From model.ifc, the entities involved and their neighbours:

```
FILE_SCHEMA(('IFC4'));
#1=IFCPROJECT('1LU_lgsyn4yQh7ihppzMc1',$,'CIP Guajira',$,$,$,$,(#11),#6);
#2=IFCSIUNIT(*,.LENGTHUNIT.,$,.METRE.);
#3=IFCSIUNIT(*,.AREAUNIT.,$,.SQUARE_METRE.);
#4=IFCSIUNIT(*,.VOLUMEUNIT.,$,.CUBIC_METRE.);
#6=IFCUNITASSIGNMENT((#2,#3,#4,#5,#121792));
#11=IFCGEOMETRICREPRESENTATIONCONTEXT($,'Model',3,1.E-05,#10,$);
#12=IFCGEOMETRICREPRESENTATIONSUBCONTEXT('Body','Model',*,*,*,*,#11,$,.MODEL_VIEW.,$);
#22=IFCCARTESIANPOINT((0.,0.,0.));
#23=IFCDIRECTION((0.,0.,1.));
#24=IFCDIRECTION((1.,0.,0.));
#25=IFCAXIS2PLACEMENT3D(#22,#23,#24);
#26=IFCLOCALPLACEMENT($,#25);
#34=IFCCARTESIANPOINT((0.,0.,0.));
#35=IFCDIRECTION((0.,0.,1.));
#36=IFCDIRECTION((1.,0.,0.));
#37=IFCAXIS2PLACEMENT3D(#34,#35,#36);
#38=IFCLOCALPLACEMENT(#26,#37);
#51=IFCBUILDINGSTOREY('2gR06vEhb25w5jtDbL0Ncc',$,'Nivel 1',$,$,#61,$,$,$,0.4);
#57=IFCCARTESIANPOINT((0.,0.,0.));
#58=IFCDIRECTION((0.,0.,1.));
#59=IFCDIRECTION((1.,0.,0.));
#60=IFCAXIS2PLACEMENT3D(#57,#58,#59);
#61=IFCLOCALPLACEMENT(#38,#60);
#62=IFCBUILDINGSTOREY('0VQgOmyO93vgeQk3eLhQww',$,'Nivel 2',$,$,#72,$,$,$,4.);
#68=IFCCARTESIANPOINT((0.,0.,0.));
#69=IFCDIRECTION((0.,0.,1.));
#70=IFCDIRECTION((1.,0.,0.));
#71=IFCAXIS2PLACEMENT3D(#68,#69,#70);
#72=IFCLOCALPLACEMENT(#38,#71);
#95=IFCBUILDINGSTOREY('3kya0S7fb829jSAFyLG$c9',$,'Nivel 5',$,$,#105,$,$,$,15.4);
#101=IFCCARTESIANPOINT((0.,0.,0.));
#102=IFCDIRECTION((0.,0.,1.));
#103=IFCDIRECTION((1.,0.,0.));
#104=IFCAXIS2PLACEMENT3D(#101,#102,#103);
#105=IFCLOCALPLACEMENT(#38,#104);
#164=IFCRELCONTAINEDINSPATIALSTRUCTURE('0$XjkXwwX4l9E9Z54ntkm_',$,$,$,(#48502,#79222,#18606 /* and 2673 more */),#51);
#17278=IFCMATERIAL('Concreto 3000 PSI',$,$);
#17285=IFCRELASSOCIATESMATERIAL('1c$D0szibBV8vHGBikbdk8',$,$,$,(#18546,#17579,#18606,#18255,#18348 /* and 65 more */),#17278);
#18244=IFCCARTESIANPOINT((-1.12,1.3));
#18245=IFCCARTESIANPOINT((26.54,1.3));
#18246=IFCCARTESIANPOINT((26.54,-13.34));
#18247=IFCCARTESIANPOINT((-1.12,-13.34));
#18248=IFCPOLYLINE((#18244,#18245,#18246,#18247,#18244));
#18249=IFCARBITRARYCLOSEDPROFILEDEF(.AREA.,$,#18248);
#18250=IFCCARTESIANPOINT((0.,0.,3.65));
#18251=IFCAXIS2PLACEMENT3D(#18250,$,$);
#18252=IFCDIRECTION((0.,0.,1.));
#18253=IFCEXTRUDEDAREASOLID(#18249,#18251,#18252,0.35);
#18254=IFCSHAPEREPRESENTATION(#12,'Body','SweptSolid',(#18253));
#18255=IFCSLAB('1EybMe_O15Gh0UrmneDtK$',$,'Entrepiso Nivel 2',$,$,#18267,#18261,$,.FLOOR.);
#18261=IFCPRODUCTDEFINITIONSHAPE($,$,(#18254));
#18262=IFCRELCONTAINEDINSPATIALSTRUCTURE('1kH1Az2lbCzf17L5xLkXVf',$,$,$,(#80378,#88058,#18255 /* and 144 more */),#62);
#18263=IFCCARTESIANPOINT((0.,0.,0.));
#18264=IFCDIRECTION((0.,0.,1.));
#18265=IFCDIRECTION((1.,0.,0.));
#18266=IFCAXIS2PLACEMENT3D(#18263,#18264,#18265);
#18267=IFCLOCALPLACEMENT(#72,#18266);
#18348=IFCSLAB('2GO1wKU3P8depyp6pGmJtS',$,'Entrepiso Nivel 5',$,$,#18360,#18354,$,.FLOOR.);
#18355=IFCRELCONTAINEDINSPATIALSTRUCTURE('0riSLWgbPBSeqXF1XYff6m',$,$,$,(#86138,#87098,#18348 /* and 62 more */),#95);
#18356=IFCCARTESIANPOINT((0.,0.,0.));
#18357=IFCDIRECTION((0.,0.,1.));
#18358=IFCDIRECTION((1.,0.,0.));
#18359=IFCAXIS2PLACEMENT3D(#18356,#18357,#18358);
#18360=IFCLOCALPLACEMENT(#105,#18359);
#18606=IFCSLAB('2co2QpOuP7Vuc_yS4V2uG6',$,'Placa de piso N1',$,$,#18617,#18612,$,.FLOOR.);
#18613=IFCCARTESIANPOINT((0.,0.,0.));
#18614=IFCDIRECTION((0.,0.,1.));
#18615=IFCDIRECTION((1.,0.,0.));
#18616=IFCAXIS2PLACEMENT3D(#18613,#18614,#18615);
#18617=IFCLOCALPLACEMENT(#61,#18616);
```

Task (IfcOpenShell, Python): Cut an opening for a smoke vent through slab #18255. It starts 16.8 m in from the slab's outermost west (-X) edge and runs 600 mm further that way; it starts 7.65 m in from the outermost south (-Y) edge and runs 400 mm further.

```python
import numpy as np
import ifcopenshell
import ifcopenshell.api.feature
import ifcopenshell.api.geometry
import ifcopenshell.api.root
import ifcopenshell.geom
import ifcopenshell.util.placement
import ifcopenshell.util.representation
import ifcopenshell.util.shape
import ifcopenshell.util.unit

model = ifcopenshell.open("model.ifc")
unit_scale = ifcopenshell.util.unit.calculate_unit_scale(model)
settings = ifcopenshell.geom.settings()


def volume(element):
    """Net volume in cubic metres, openings subtracted."""
    shape = ifcopenshell.geom.create_shape(settings, element)
    return ifcopenshell.util.shape.get_volume(shape.geometry)


slab = model.by_id(18255)
before = volume(slab)

# Extent in the slab's own axes, in metres. The edges named are its -X and -Y sides.
slab_shape = ifcopenshell.geom.create_shape(settings, slab)
vertices = ifcopenshell.util.shape.get_vertices(slab_shape.geometry)
x_min, y_min, bottom = vertices.min(axis=0)
top = vertices[:, 2].max()

opening = ifcopenshell.api.root.create_entity(model, ifc_class="IfcOpeningElement", name="Smoke vent opening", predefined_type="OPENING")
context = ifcopenshell.util.representation.get_context(model, "Model", "Body", "MODEL_VIEW")
width, depth = 0.6, 0.4
outline = [(0.0, 0.0), (width, 0.0), (width, depth), (0.0, depth), (0.0, 0.0)]
# Overshoot both faces by 50 mm so the cut is clean.
shape = ifcopenshell.api.geometry.add_slab_representation(
    model, context=context, depth=top - bottom + 0.1, polyline=outline
)
ifcopenshell.api.geometry.assign_representation(model, product=opening, representation=shape)

matrix = ifcopenshell.util.placement.get_local_placement(slab.ObjectPlacement)
matrix[:, 3] = matrix @ np.append(np.array([x_min + 16.8, y_min + 7.65, bottom - 0.05]) / unit_scale, 1.0)
ifcopenshell.api.geometry.edit_object_placement(model, product=opening, matrix=matrix, is_si=False)
ifcopenshell.api.feature.add_feature(model, feature=opening, element=slab)

after = volume(slab)

print(f"slab volume {before:.3f} -> {after:.3f} m3")

model.write("model_edited.ifc")
```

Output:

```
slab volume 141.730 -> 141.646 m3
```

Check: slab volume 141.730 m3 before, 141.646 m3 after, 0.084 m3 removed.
